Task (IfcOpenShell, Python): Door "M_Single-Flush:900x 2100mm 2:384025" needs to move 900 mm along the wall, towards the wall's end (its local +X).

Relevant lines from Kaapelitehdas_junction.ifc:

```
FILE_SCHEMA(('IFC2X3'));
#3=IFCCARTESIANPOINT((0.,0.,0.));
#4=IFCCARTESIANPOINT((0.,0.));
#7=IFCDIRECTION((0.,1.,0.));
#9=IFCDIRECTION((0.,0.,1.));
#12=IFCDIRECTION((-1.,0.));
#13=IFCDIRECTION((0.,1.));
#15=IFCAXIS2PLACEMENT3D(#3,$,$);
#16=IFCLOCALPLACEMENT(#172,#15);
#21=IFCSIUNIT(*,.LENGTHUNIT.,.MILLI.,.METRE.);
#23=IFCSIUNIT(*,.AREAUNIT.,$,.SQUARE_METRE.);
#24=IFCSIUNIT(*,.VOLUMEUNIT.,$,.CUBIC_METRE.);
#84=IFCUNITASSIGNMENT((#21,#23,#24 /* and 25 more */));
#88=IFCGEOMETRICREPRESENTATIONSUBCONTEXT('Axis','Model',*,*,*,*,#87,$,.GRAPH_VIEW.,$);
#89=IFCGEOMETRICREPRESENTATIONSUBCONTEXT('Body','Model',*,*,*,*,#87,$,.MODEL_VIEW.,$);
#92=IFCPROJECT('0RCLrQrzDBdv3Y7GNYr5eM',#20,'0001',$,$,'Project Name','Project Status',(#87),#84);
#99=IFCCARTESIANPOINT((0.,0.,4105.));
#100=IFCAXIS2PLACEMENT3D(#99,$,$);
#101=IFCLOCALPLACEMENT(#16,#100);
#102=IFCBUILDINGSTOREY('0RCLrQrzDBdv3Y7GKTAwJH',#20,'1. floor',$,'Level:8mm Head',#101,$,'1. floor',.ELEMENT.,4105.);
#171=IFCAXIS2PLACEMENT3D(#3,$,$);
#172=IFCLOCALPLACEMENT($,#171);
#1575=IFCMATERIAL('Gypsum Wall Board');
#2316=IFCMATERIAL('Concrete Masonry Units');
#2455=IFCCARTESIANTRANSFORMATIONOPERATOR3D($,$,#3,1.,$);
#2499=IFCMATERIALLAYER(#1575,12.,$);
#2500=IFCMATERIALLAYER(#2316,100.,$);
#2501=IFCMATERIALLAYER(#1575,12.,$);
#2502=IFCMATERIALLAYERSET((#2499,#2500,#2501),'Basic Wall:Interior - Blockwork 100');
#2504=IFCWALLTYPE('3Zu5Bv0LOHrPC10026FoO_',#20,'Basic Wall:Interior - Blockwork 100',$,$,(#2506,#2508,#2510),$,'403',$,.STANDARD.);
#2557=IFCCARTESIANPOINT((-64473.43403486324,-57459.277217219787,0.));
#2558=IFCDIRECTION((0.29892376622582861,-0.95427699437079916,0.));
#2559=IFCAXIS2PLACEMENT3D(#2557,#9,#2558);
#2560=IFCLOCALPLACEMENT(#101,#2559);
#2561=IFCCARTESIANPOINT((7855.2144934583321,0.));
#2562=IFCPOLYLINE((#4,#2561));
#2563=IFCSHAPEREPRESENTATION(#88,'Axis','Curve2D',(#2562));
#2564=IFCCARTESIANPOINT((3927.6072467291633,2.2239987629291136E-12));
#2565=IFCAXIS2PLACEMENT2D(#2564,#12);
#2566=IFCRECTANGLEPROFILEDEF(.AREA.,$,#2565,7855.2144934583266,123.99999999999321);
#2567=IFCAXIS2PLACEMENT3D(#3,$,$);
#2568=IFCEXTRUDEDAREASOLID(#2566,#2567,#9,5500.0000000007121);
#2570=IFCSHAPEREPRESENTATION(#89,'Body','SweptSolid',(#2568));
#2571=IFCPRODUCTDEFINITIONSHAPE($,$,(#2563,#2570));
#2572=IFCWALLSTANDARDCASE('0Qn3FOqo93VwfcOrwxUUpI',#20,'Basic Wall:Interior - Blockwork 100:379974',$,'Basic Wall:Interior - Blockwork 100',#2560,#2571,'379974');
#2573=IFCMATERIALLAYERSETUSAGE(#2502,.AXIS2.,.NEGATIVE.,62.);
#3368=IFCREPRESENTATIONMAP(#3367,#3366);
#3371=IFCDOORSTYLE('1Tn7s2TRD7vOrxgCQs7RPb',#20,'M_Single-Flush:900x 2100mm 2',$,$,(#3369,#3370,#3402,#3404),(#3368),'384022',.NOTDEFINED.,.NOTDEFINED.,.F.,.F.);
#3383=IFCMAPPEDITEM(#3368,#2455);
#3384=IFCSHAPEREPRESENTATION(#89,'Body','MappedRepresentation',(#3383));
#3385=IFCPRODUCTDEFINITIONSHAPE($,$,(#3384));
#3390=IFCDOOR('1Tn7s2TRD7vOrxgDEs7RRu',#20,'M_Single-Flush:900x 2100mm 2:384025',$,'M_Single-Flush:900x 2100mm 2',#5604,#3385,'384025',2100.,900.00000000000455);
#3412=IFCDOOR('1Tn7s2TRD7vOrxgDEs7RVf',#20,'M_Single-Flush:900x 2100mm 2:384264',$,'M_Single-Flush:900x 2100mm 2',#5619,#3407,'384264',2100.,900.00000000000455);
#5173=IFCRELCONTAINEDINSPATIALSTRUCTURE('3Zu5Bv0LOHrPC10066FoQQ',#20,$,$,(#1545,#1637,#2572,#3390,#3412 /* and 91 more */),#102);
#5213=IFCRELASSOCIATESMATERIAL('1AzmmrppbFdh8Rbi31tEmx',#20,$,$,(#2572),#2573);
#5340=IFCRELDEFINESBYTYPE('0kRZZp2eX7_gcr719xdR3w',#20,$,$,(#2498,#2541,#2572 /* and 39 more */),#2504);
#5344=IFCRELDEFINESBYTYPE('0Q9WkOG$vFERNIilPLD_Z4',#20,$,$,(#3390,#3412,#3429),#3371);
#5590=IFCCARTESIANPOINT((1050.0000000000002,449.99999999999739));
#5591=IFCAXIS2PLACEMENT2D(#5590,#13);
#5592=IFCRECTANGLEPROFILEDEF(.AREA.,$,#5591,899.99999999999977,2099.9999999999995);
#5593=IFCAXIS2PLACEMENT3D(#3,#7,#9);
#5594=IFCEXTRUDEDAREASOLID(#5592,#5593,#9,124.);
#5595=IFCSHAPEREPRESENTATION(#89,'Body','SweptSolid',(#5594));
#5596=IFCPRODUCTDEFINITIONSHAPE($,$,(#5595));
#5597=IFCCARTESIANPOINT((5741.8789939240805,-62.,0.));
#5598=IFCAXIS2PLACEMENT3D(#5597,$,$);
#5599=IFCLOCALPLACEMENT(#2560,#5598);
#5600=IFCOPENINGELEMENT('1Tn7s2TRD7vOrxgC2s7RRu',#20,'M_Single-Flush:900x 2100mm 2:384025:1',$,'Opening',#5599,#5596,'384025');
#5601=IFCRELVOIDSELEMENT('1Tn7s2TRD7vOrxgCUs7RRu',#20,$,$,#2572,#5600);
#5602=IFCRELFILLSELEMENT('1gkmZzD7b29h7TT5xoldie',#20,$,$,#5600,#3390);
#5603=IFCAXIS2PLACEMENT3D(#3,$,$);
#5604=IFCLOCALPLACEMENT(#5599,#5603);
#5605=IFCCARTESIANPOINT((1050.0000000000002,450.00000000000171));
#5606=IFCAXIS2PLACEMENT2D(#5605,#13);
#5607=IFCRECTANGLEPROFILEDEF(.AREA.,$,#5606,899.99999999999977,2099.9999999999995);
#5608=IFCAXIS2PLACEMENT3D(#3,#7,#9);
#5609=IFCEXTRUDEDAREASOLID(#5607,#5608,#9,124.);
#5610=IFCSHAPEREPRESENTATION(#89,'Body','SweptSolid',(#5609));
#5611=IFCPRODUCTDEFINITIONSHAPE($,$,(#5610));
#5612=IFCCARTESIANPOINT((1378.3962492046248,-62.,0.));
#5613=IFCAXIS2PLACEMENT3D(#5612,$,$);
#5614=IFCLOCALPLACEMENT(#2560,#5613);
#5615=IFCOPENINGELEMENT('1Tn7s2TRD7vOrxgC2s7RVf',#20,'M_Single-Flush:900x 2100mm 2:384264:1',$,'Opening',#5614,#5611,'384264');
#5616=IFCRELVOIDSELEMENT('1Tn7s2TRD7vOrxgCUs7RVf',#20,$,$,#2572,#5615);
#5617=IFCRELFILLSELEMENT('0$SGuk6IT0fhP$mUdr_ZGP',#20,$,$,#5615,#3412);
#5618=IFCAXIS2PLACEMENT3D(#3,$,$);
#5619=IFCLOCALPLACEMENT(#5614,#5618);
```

```python
import ifcopenshell
import ifcopenshell.api.geometry
import ifcopenshell.util.placement
import ifcopenshell.util.unit

model = ifcopenshell.open("Kaapelitehdas_junction.ifc")
unit_scale = ifcopenshell.util.unit.calculate_unit_scale(model)

door = model.by_guid("1Tn7s2TRD7vOrxgDEs7RRu")
opening = door.FillsVoids[0].RelatingOpeningElement
wall = opening.VoidsElements[0].RelatingBuildingElement

wall_matrix = ifcopenshell.util.placement.get_local_placement(wall.ObjectPlacement)
shift = wall_matrix[:3, 0] * 0.9 / unit_scale
before = ifcopenshell.util.placement.get_local_placement(door.ObjectPlacement)[:3, 3].copy()

# The door is placed relative to its opening, so it follows when the opening moves.
matrix = ifcopenshell.util.placement.get_local_placement(opening.ObjectPlacement)
matrix[:3, 3] += shift
ifcopenshell.api.geometry.edit_object_placement(
    model, product=opening, matrix=matrix, is_si=False, should_transform_children=True
)

after = ifcopenshell.util.placement.get_local_placement(door.ObjectPlacement)[:3, 3]
print("door moved by", (after - before).round(3) + 0.0)

model.write("Kaapelitehdas_junction_edited.ifc")
```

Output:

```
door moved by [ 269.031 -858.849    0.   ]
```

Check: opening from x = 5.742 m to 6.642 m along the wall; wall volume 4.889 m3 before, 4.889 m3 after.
